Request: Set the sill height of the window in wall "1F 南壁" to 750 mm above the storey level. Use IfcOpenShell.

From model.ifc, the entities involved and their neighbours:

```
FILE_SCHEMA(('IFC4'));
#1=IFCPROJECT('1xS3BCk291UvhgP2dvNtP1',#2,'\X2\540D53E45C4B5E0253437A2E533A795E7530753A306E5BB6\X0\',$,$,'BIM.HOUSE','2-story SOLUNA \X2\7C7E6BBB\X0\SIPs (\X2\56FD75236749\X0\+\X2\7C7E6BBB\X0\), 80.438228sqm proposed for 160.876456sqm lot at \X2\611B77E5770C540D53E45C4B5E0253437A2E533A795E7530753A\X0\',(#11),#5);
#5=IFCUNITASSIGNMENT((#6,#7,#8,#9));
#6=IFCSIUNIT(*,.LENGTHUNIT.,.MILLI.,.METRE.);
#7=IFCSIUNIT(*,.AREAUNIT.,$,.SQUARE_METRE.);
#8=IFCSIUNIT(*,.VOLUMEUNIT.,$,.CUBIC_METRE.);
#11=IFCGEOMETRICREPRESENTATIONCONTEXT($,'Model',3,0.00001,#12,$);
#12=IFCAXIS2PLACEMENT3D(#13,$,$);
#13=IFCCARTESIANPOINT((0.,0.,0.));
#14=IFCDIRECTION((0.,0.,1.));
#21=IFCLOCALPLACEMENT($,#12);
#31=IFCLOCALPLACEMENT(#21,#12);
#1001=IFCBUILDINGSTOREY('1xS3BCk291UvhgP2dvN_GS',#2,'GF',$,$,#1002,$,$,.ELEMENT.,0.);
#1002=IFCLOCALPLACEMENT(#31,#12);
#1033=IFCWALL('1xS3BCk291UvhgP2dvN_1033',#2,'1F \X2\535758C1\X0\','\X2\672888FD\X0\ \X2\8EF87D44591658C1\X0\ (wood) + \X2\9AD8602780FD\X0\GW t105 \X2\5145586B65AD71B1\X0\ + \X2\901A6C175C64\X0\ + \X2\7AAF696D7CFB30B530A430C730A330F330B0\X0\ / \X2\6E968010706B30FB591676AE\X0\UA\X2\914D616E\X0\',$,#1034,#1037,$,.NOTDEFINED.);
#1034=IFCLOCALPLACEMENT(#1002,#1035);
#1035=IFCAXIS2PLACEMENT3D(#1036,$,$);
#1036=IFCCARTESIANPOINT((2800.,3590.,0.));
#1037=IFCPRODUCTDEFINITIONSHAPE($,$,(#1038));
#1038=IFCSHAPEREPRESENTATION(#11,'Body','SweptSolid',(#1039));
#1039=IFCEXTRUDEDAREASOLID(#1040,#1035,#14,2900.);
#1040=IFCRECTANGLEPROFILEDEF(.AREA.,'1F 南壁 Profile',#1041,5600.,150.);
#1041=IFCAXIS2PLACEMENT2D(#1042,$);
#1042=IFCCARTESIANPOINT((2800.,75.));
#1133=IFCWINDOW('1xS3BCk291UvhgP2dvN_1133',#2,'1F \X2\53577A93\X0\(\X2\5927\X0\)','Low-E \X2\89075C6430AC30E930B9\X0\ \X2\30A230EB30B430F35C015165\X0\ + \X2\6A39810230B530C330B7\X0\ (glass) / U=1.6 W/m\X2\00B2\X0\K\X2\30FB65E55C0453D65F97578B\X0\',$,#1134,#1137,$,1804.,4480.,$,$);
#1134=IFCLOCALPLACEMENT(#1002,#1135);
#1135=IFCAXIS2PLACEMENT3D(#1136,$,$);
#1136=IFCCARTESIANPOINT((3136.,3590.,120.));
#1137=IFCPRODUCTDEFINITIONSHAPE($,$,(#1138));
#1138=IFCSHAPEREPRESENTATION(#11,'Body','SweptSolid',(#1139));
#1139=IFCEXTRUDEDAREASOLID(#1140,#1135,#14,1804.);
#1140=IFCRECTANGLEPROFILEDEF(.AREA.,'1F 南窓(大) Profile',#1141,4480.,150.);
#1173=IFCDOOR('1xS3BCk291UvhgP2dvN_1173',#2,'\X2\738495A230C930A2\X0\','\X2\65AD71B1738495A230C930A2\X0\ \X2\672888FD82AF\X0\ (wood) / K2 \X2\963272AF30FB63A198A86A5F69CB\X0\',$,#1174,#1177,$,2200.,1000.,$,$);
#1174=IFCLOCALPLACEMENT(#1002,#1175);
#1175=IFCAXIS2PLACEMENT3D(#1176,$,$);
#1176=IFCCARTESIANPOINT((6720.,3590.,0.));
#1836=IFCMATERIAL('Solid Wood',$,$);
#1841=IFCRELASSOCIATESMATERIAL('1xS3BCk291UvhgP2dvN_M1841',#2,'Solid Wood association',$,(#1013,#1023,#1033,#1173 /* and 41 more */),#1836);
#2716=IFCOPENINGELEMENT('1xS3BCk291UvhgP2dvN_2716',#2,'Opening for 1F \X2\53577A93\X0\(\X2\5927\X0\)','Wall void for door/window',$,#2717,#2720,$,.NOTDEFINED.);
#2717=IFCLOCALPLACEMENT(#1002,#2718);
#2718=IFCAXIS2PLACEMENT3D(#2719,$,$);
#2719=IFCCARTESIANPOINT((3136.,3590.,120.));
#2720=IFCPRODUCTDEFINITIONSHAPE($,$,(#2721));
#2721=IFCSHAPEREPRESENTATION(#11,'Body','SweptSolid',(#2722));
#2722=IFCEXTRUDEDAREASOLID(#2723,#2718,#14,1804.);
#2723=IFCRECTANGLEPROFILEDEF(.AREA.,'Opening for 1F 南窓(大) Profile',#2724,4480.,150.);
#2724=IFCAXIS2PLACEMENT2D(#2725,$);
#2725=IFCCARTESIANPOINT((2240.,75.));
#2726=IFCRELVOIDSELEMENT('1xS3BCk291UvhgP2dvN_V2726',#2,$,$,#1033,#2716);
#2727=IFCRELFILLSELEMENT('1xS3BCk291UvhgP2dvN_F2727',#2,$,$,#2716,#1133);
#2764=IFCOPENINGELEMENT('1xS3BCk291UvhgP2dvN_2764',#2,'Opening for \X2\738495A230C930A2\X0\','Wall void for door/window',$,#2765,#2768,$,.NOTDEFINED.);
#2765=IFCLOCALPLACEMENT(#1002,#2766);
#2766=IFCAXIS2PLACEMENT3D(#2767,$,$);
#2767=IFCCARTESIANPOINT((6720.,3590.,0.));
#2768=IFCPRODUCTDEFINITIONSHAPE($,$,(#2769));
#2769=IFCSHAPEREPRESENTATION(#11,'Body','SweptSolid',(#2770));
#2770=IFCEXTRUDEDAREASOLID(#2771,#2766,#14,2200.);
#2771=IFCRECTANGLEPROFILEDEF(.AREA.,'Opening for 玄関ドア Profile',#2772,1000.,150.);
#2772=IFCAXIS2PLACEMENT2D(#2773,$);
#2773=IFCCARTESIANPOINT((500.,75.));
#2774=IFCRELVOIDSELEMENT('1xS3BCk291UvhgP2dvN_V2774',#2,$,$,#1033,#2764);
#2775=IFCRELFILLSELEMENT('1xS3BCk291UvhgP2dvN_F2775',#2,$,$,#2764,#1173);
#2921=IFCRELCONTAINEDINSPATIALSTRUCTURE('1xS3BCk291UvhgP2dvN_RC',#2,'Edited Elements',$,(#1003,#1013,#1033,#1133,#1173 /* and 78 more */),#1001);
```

```python
import numpy as np
import ifcopenshell
import ifcopenshell.api.geometry
import ifcopenshell.geom
import ifcopenshell.util.element
import ifcopenshell.util.placement
import ifcopenshell.util.shape
import ifcopenshell.util.unit

model = ifcopenshell.open("model.ifc")
unit_scale = ifcopenshell.util.unit.calculate_unit_scale(model)

window = model.by_id(1133)
opening = window.FillsVoids[0].RelatingOpeningElement
storey = ifcopenshell.util.element.get_container(window, ifc_class="IfcBuildingStorey")
level = ifcopenshell.util.placement.get_local_placement(storey.ObjectPlacement)[2, 3]

# The opening's origin need not be at the sill, so measure its lowest point.
shape = ifcopenshell.geom.create_shape(ifcopenshell.geom.settings(), opening)
bottom = ifcopenshell.util.shape.get_shape_bottom_elevation(shape, shape.geometry) / unit_scale
dz = level + 750.0 - bottom

shift = np.array([0.0, 0.0, dz])
# The window is not placed relative to its opening, so move both.
for product in (opening, window):
    matrix = ifcopenshell.util.placement.get_local_placement(product.ObjectPlacement)
    matrix[:3, 3] += shift
    ifcopenshell.api.geometry.edit_object_placement(model, product=product, matrix=matrix, is_si=False)

print(f"moved by {dz * unit_scale:+.3f} m")

model.write("model_rev.ifc")
```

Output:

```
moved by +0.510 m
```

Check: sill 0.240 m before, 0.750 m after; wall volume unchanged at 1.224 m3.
